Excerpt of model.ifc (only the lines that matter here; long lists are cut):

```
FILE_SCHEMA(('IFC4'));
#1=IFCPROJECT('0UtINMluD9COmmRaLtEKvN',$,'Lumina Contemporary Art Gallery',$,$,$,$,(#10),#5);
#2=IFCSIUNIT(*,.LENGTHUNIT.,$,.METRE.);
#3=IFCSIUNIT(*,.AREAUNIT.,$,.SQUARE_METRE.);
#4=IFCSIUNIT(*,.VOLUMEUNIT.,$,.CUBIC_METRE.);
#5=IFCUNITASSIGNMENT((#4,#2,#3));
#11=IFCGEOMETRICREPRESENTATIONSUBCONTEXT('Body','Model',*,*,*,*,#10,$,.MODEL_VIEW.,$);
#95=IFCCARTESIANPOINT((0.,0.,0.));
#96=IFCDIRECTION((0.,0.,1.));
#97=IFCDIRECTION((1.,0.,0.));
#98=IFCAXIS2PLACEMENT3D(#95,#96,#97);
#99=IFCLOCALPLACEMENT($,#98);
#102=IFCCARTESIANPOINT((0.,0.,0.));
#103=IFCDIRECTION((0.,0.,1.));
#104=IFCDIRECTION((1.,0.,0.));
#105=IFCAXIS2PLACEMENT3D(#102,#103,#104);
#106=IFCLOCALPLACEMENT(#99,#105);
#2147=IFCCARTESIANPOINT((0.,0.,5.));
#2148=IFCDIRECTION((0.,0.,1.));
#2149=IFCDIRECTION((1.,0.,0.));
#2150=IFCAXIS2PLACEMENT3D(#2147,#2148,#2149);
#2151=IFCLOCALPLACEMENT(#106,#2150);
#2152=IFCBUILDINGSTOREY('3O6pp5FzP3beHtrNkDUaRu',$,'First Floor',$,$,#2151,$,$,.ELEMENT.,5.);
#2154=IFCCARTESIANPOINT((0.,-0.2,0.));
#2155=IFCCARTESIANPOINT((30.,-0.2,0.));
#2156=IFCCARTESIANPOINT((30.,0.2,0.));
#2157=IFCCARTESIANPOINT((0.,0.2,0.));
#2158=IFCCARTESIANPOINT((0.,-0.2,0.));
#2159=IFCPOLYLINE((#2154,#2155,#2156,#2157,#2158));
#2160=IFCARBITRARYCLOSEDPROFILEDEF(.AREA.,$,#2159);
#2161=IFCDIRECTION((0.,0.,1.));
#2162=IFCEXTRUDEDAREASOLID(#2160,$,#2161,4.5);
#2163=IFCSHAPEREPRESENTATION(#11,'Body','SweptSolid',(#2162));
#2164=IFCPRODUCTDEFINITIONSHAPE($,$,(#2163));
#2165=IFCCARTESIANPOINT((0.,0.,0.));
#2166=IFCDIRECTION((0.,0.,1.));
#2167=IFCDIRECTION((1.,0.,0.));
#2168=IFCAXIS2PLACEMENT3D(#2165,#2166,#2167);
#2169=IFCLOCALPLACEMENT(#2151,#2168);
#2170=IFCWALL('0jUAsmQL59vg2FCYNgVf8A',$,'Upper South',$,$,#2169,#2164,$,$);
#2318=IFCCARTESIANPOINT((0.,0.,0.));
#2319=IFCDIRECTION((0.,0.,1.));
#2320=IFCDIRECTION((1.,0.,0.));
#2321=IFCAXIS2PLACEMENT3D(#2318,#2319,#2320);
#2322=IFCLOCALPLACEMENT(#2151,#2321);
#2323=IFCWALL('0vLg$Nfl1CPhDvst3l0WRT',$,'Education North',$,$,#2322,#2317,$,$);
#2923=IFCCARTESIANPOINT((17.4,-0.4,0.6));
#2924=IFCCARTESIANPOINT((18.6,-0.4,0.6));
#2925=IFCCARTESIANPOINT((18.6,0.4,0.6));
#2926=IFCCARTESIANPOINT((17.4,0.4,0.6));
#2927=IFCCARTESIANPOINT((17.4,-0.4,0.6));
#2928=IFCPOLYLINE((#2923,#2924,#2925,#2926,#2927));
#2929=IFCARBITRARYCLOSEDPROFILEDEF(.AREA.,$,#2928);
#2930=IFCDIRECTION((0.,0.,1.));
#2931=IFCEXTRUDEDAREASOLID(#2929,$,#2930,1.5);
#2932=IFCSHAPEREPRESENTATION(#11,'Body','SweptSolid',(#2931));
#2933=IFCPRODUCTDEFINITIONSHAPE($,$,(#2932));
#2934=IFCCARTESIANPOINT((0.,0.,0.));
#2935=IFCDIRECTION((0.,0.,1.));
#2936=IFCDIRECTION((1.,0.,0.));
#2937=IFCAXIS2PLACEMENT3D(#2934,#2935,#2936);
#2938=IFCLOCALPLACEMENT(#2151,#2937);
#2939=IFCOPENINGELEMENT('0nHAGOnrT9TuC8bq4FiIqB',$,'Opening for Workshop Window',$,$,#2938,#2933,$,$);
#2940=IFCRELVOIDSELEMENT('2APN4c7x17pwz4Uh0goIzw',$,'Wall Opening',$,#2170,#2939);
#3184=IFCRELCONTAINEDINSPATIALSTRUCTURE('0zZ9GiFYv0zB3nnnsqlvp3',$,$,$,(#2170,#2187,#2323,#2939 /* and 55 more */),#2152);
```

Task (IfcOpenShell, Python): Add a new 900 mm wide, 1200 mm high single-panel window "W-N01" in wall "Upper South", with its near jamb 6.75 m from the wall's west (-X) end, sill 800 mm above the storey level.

```python
import numpy as np
import ifcopenshell
import ifcopenshell.api.feature
import ifcopenshell.api.geometry
import ifcopenshell.api.root
import ifcopenshell.api.spatial
import ifcopenshell.geom
import ifcopenshell.util.element
import ifcopenshell.util.placement
import ifcopenshell.util.representation
import ifcopenshell.util.shape
import ifcopenshell.util.unit

model = ifcopenshell.open("model.ifc")
unit_scale = ifcopenshell.util.unit.calculate_unit_scale(model)
settings = ifcopenshell.geom.settings()


def volume(element):
    """Net volume in cubic metres, openings subtracted."""
    shape = ifcopenshell.geom.create_shape(settings, element)
    return ifcopenshell.util.shape.get_volume(shape.geometry)


wall = model.by_guid("0jUAsmQL59vg2FCYNgVf8A")
storey = ifcopenshell.util.element.get_container(wall, ifc_class="IfcBuildingStorey")
context = ifcopenshell.util.representation.get_context(model, "Model", "Body", "MODEL_VIEW")
before = volume(wall)

width, height, from_end, sill = 0.9, 1.2, 6.75, 0.8  # metres

# The wall runs along its own X axis, and the end named is its -X end.
wall_shape = ifcopenshell.geom.create_shape(settings, wall)
x, y, z = ifcopenshell.util.shape.get_vertices(wall_shape.geometry).T
start = x.min() + from_end
face, thickness = float(y.min()), float(y.max() - y.min())
wall_matrix = ifcopenshell.util.placement.get_local_placement(wall.ObjectPlacement)
level = ifcopenshell.util.placement.get_local_placement(storey.ObjectPlacement)[2, 3]


def in_wall(x, y):
    """Placement at x, y metres in the wall's axes, at sill height."""
    matrix = wall_matrix.copy()
    matrix[:, 3] = wall_matrix @ np.array([x / unit_scale, y / unit_scale, 0.0, 1.0])
    matrix[2, 3] = level + sill / unit_scale
    return matrix


# Opening: a box that overshoots both wall faces by 50 mm.
opening = ifcopenshell.api.root.create_entity(model, ifc_class="IfcOpeningElement", predefined_type="OPENING")
box = ifcopenshell.api.geometry.add_wall_representation(
    model, context=context, length=width, height=height, thickness=thickness + 0.1
)
ifcopenshell.api.geometry.assign_representation(model, product=opening, representation=box)
ifcopenshell.api.geometry.edit_object_placement(model, product=opening, matrix=in_wall(start, face - 0.05), is_si=False)
ifcopenshell.api.feature.add_feature(model, feature=opening, element=wall)

window = ifcopenshell.api.root.create_entity(model, ifc_class="IfcWindow", name="W-N01", predefined_type="WINDOW")
window.OverallWidth, window.OverallHeight = width / unit_scale, height / unit_scale
window.PartitioningType = "SINGLE_PANEL"
body = ifcopenshell.api.geometry.add_window_representation(
    model,
    context=context,
    overall_width=window.OverallWidth,
    overall_height=window.OverallHeight,
    partition_type="SINGLE_PANEL",
)
ifcopenshell.api.geometry.assign_representation(model, product=window, representation=body)
ifcopenshell.api.spatial.assign_container(model, products=[window], relating_structure=storey)
ifcopenshell.api.feature.add_filling(model, opening=opening, element=window)

# Centre the window in the wall's thickness.
ifcopenshell.api.geometry.edit_object_placement(model, product=window, matrix=in_wall(start, face), is_si=False)
window_shape = ifcopenshell.geom.create_shape(settings, window)
depth = ifcopenshell.util.shape.get_vertices(window_shape.geometry)[:, 1]
offset = face + thickness / 2 - (depth.min() + depth.max()) / 2
ifcopenshell.api.geometry.edit_object_placement(model, product=window, matrix=in_wall(start, offset), is_si=False)

after = volume(wall)

print(f"wall volume {before:.3f} -> {after:.3f} m3")

model.write("model_edited.ifc")
```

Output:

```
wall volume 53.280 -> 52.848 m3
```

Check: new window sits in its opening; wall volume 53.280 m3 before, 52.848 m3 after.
